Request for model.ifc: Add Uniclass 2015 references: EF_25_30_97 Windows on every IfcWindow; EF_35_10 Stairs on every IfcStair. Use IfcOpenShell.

First a look at what the model holds.

```python
import ifcopenshell

model = ifcopenshell.open("model.ifc")
print(model.schema)
print("classifications:", [c.Name for c in model.by_type("IfcClassification")])
for ifc_class in ("IfcDoor", "IfcRoof", "IfcStair", "IfcWall", "IfcWindow"):
    print(ifc_class, len(model.by_type(ifc_class)))
```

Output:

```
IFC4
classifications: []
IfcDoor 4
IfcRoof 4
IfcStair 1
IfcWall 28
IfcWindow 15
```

```python
import ifcopenshell
import ifcopenshell.api.classification

model = ifcopenshell.open("model.ifc")

system = ifcopenshell.api.classification.add_classification(model, classification="Uniclass 2015")

codes = {
    "IfcWindow": ("EF_25_30_97", "Windows"),
    "IfcStair": ("EF_35_10", "Stairs"),
}
for ifc_class, (code, name) in codes.items():
    products = model.by_type(ifc_class)
    ifcopenshell.api.classification.add_reference(
        model, products=products, classification=system, identification=code, name=name
    )
    print(code, len(products))

model.write("model_edited.ifc")
```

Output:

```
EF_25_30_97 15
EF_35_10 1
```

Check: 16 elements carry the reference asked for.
